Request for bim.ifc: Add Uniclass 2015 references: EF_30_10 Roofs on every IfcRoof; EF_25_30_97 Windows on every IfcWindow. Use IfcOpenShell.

First a look at what the model holds.

```python
import ifcopenshell

model = ifcopenshell.open("bim.ifc")
print(model.schema)
print("classifications:", [c.Name for c in model.by_type("IfcClassification")])
for ifc_class in ("IfcDoor", "IfcRoof", "IfcStair", "IfcWall", "IfcWindow"):
    print(ifc_class, len(model.by_type(ifc_class)))
```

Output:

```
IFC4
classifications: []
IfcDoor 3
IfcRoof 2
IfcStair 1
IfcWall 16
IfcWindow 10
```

```python
import ifcopenshell
import ifcopenshell.api.classification

model = ifcopenshell.open("bim.ifc")

system = ifcopenshell.api.classification.add_classification(model, classification="Uniclass 2015")

codes = {
    "IfcRoof": ("EF_30_10", "Roofs"),
    "IfcWindow": ("EF_25_30_97", "Windows"),
}
for ifc_class, (code, name) in codes.items():
    products = model.by_type(ifc_class)
    ifcopenshell.api.classification.add_reference(
        model, products=products, classification=system, identification=code, name=name
    )
    print(code, len(products))

model.write("bim_edited.ifc")
```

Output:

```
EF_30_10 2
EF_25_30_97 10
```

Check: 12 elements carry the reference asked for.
